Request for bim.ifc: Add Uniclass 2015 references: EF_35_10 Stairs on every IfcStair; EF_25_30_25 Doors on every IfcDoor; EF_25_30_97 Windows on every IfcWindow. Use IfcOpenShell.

First a look at what the model holds.

```python
import ifcopenshell

model = ifcopenshell.open("bim.ifc")
print(model.schema)
print("classifications:", [c.Name for c in model.by_type("IfcClassification")])
for ifc_class in ("IfcDoor", "IfcRoof", "IfcStair", "IfcWall", "IfcWindow"):
    print(ifc_class, len(model.by_type(ifc_class)))
```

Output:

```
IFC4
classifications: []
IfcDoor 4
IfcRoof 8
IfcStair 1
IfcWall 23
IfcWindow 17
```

```python
import ifcopenshell
import ifcopenshell.api.classification

model = ifcopenshell.open("bim.ifc")

system = ifcopenshell.api.classification.add_classification(model, classification="Uniclass 2015")

codes = {
    "IfcStair": ("EF_35_10", "Stairs"),
    "IfcDoor": ("EF_25_30_25", "Doors"),
    "IfcWindow": ("EF_25_30_97", "Windows"),
}
for ifc_class, (code, name) in codes.items():
    products = model.by_type(ifc_class)
    ifcopenshell.api.classification.add_reference(
        model, products=products, classification=system, identification=code, name=name
    )
    print(code, len(products))

model.write("bim_edited.ifc")
```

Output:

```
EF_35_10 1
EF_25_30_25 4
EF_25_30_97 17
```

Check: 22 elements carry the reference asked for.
